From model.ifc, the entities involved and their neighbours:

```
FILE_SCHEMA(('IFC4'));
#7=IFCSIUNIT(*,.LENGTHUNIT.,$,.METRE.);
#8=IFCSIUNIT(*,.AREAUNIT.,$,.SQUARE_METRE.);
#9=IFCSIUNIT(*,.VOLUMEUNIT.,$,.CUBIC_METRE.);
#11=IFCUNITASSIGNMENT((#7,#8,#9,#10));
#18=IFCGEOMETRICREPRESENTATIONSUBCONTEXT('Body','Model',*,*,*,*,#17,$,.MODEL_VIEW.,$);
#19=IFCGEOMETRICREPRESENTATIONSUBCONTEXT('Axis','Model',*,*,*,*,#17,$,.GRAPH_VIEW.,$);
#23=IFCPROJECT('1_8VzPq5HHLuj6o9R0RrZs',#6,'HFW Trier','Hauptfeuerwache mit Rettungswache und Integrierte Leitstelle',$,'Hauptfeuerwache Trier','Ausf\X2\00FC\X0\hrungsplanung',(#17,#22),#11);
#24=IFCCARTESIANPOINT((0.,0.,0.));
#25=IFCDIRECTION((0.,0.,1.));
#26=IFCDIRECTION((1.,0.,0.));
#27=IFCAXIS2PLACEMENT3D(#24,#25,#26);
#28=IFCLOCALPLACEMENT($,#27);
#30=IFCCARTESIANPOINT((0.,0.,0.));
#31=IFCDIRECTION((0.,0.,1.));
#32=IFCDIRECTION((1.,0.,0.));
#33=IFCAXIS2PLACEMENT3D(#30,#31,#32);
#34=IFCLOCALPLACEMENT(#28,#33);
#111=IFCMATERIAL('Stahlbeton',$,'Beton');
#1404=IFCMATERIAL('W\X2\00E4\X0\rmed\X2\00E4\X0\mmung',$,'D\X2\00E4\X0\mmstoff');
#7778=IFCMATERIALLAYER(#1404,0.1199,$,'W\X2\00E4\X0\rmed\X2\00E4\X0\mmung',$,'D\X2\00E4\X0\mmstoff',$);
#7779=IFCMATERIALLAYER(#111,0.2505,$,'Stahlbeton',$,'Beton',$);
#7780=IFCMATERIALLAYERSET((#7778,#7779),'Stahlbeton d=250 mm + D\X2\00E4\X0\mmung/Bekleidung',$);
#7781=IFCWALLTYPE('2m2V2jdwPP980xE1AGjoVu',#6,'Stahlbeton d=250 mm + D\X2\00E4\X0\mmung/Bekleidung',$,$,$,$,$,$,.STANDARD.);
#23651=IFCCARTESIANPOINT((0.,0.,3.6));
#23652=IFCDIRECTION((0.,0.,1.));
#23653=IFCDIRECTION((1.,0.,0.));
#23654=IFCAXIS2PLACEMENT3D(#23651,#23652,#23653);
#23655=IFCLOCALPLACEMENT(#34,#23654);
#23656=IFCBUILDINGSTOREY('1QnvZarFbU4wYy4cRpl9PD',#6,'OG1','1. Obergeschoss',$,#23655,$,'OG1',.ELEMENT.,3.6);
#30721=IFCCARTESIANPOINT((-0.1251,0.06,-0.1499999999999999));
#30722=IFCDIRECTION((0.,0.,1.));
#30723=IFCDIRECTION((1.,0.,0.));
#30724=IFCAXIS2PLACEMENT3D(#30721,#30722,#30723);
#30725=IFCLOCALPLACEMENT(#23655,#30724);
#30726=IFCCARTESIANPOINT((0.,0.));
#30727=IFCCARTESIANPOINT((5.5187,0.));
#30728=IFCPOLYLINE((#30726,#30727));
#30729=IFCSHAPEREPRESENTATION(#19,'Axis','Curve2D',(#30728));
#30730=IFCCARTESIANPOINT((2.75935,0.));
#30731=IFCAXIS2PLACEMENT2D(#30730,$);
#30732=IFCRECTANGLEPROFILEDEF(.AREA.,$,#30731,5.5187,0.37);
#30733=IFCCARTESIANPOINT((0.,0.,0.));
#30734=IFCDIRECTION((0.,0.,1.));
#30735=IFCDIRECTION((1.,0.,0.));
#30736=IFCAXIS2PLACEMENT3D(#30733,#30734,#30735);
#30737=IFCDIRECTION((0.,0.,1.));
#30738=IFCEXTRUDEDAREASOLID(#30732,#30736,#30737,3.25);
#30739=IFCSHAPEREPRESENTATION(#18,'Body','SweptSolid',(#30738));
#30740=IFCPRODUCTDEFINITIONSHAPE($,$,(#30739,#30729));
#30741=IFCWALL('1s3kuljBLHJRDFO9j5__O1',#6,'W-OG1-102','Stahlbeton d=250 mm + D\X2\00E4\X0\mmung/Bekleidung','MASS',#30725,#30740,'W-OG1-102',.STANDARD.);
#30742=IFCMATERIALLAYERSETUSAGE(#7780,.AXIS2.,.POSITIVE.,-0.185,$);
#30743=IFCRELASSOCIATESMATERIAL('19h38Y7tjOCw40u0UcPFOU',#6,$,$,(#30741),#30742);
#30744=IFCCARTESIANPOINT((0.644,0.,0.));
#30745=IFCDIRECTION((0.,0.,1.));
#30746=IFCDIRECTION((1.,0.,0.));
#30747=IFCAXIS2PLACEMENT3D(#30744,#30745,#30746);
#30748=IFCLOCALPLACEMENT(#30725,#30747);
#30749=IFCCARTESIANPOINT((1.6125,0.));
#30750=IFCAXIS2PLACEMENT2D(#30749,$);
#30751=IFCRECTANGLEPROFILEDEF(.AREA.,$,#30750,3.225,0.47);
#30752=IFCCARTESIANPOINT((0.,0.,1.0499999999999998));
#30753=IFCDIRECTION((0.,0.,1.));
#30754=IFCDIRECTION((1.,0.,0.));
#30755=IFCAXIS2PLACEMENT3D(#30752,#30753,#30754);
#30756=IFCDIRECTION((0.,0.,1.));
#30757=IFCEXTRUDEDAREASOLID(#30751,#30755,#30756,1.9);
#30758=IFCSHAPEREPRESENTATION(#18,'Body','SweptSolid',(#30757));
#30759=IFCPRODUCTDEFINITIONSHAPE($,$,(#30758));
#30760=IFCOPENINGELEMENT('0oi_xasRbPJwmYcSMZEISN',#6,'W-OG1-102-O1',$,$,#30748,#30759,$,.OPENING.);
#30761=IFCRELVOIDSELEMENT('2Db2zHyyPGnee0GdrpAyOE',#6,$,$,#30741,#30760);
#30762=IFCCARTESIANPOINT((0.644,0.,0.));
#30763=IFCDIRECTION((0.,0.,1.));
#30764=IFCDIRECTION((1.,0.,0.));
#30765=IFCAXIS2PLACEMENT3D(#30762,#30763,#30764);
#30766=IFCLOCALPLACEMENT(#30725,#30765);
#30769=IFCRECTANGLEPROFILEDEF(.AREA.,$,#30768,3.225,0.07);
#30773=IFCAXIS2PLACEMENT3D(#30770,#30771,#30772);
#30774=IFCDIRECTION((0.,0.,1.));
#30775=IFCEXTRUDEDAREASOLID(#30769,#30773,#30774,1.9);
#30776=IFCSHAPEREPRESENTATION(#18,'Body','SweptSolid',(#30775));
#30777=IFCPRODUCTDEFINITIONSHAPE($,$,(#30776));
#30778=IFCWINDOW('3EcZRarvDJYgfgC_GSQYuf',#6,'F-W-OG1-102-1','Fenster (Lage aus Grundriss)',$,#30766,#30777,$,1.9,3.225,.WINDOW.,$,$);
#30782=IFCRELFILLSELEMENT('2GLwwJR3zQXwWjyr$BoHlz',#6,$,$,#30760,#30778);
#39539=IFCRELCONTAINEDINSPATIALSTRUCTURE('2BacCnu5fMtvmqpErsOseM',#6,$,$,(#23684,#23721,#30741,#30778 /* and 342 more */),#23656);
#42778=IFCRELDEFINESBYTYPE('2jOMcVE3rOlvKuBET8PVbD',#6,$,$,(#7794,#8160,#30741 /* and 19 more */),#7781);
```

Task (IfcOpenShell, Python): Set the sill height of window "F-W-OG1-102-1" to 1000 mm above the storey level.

```python
import numpy as np
import ifcopenshell
import ifcopenshell.api.geometry
import ifcopenshell.geom
import ifcopenshell.util.element
import ifcopenshell.util.placement
import ifcopenshell.util.shape
import ifcopenshell.util.unit

model = ifcopenshell.open("model.ifc")
unit_scale = ifcopenshell.util.unit.calculate_unit_scale(model)

window = model.by_guid("3EcZRarvDJYgfgC_GSQYuf")
opening = window.FillsVoids[0].RelatingOpeningElement
storey = ifcopenshell.util.element.get_container(window, ifc_class="IfcBuildingStorey")
level = ifcopenshell.util.placement.get_local_placement(storey.ObjectPlacement)[2, 3]

# The opening's origin need not be at the sill, so measure its lowest point.
shape = ifcopenshell.geom.create_shape(ifcopenshell.geom.settings(), opening)
bottom = ifcopenshell.util.shape.get_shape_bottom_elevation(shape, shape.geometry) / unit_scale
dz = level + 1.0 - bottom

shift = np.array([0.0, 0.0, dz])
# The window is not placed relative to its opening, so move both.
for product in (opening, window):
    matrix = ifcopenshell.util.placement.get_local_placement(product.ObjectPlacement)
    matrix[:3, 3] += shift
    ifcopenshell.api.geometry.edit_object_placement(model, product=product, matrix=matrix, is_si=False)

print(f"moved by {dz * unit_scale:+.3f} m")

model.write("model_rev.ifc")
```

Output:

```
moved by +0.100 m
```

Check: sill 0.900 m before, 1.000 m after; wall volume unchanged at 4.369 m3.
